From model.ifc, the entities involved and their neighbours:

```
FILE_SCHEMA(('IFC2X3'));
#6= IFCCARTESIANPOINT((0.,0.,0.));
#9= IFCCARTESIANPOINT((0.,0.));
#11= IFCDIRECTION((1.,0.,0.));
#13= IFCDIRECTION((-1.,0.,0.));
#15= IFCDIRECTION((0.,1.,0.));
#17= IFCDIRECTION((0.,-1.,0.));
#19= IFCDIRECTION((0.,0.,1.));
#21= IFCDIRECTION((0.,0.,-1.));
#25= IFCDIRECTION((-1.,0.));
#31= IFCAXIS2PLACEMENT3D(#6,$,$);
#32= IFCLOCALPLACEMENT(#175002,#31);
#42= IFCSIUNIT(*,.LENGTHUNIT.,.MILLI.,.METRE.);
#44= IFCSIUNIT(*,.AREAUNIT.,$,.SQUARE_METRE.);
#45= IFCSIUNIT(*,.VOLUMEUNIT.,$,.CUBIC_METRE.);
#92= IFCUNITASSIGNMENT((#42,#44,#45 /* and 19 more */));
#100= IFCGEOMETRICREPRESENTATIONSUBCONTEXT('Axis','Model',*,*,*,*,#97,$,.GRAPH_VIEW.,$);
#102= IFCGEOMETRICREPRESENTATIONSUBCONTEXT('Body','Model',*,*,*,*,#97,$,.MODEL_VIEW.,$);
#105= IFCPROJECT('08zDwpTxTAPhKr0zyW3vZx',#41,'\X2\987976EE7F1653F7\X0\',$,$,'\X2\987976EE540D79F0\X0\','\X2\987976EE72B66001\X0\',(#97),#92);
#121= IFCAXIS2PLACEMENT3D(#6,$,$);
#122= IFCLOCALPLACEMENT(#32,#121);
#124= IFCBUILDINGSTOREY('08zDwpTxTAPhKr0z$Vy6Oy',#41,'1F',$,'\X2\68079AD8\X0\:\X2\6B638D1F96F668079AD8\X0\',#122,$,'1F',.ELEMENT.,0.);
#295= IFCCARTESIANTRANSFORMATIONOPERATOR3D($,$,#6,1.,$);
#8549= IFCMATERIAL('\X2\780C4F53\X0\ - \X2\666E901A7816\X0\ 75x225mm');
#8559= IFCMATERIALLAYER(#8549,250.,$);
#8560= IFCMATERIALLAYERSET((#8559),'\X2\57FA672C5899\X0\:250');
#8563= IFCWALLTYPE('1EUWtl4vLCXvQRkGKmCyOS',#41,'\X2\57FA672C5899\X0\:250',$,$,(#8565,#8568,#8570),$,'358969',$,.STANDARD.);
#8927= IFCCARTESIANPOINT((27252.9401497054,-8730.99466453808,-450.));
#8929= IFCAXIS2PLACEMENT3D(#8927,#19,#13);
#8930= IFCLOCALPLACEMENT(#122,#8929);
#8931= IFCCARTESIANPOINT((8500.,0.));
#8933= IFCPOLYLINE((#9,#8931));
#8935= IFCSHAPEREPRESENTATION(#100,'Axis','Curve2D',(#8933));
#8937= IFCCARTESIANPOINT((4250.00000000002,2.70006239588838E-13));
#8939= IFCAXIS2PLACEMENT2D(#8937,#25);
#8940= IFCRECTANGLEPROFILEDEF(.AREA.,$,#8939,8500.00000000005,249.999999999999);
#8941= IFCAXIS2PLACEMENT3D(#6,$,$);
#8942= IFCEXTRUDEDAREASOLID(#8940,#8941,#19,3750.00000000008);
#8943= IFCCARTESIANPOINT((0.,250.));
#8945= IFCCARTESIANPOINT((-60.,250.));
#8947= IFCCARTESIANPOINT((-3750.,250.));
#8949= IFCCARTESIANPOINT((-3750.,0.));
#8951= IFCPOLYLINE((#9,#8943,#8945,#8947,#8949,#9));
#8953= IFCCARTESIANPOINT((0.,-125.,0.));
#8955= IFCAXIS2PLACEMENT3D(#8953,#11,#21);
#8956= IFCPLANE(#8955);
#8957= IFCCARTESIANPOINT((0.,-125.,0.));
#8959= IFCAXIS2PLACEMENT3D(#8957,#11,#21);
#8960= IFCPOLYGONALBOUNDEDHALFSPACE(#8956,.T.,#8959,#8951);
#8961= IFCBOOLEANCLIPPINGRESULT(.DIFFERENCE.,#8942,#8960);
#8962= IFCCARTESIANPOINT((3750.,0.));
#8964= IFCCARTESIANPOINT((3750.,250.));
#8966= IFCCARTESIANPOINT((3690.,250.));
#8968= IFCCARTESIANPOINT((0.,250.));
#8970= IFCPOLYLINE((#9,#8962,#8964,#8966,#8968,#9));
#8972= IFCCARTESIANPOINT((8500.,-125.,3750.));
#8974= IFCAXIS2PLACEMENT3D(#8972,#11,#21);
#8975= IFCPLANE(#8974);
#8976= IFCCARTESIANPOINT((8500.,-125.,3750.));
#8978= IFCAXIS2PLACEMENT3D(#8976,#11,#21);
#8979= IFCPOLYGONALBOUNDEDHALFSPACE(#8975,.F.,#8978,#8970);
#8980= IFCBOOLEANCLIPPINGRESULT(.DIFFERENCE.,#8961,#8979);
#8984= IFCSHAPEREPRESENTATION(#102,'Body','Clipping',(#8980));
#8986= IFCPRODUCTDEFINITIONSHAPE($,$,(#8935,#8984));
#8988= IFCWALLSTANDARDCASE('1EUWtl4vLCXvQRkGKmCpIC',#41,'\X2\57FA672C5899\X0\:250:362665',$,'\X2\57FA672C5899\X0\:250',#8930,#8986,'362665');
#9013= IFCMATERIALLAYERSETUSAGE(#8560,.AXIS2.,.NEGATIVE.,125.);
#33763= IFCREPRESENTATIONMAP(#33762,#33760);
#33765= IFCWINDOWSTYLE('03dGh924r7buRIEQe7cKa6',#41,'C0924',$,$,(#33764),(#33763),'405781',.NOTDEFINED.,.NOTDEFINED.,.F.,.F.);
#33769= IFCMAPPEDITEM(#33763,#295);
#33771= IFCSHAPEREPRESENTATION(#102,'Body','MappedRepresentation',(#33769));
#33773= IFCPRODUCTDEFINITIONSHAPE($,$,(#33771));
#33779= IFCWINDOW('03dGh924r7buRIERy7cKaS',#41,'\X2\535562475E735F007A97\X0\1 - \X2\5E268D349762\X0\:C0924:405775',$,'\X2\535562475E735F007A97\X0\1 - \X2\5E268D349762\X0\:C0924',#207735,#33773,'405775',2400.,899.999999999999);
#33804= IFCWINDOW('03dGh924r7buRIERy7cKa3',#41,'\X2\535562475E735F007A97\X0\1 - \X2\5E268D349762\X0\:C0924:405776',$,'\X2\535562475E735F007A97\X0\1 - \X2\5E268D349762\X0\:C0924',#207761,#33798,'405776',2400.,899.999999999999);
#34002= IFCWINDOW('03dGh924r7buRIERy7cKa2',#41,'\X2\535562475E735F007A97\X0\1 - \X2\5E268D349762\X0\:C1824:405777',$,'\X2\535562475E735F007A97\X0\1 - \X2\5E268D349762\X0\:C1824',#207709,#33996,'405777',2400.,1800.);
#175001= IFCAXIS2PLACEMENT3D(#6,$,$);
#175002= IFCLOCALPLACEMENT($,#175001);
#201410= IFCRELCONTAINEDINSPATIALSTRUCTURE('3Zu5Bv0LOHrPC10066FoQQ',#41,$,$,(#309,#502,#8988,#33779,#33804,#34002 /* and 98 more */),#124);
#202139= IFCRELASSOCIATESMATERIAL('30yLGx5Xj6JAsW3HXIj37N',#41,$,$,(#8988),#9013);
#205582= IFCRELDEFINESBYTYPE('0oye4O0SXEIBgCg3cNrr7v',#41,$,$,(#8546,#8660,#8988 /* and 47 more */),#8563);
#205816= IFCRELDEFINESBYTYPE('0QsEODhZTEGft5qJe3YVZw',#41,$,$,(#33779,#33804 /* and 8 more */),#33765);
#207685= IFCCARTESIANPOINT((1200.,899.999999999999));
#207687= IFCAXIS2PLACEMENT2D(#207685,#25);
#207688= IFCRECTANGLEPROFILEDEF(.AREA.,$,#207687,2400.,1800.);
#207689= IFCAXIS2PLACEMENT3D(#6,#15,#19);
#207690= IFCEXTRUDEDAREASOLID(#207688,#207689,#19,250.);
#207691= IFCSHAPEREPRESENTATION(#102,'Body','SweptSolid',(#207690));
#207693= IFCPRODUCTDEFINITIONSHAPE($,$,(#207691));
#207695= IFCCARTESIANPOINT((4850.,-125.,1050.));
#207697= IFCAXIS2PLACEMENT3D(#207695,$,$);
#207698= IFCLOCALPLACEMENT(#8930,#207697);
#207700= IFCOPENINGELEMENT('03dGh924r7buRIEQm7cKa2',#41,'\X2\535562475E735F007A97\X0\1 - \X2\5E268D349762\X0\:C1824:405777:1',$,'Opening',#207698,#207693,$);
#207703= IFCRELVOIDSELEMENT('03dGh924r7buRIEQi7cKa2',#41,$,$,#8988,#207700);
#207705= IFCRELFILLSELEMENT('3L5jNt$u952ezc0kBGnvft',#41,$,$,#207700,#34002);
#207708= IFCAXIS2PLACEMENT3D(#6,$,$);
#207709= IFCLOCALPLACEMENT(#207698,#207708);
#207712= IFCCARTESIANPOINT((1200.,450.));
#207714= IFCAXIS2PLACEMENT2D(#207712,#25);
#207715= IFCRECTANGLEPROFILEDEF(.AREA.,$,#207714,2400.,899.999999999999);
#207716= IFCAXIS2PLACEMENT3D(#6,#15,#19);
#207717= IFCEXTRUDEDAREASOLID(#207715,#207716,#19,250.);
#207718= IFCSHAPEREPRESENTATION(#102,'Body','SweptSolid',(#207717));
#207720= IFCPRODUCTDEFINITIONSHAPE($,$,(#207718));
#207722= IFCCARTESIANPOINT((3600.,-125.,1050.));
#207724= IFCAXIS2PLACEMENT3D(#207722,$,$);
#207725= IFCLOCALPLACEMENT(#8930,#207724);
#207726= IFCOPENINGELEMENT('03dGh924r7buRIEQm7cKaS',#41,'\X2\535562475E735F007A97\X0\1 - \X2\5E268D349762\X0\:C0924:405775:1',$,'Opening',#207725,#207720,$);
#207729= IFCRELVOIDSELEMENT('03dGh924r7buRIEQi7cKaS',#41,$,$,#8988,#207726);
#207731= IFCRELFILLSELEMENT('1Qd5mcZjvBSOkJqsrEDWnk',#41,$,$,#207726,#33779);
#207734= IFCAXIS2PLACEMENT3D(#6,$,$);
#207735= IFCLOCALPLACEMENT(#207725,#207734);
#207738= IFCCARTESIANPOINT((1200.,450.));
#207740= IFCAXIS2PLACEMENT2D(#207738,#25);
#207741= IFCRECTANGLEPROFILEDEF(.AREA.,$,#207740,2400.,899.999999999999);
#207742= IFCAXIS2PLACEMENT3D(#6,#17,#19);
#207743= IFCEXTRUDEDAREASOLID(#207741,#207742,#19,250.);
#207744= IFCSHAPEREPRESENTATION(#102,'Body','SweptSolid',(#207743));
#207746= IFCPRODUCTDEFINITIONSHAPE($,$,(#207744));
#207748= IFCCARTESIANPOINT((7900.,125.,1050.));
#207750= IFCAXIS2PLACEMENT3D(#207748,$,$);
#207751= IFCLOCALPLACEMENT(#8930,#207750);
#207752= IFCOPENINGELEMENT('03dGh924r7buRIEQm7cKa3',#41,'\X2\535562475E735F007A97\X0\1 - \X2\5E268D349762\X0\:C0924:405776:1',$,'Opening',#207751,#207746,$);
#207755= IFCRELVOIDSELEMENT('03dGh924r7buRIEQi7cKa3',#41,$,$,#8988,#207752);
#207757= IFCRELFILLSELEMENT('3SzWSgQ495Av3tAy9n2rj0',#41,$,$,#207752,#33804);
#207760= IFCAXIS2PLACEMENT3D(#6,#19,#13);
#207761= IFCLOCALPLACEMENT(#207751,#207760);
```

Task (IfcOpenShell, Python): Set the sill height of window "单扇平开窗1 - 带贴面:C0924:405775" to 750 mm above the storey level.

```python
import numpy as np
import ifcopenshell
import ifcopenshell.api.geometry
import ifcopenshell.geom
import ifcopenshell.util.element
import ifcopenshell.util.placement
import ifcopenshell.util.shape
import ifcopenshell.util.unit

model = ifcopenshell.open("model.ifc")
unit_scale = ifcopenshell.util.unit.calculate_unit_scale(model)

window = model.by_guid("03dGh924r7buRIERy7cKaS")
opening = window.FillsVoids[0].RelatingOpeningElement
storey = ifcopenshell.util.element.get_container(window, ifc_class="IfcBuildingStorey")
level = ifcopenshell.util.placement.get_local_placement(storey.ObjectPlacement)[2, 3]

# The opening's origin need not be at the sill, so measure its lowest point.
shape = ifcopenshell.geom.create_shape(ifcopenshell.geom.settings(), opening)
bottom = ifcopenshell.util.shape.get_shape_bottom_elevation(shape, shape.geometry) / unit_scale
dz = level + 0.75 / unit_scale - bottom

shift = np.array([0.0, 0.0, dz])
# The window is placed relative to its opening, so it follows when the opening moves.
matrix = ifcopenshell.util.placement.get_local_placement(opening.ObjectPlacement)
matrix[:3, 3] += shift
ifcopenshell.api.geometry.edit_object_placement(
    model, product=opening, matrix=matrix, is_si=False, should_transform_children=True
)

print(f"moved by {dz * unit_scale:+.3f} m")

model.write("model_updated.ifc")
```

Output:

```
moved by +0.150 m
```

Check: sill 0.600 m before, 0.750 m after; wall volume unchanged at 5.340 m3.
